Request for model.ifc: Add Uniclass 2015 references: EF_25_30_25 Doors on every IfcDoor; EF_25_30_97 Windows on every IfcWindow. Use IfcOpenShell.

First a look at what the model holds.

```python
import ifcopenshell

model = ifcopenshell.open("model.ifc")
print(model.schema)
print("classifications:", [c.Name for c in model.by_type("IfcClassification")])
for ifc_class in ("IfcDoor", "IfcRoof", "IfcStair", "IfcWall", "IfcWindow"):
    print(ifc_class, len(model.by_type(ifc_class)))
```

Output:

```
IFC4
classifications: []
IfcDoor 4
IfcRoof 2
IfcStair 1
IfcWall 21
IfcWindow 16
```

```python
import ifcopenshell
import ifcopenshell.api.classification

model = ifcopenshell.open("model.ifc")

system = ifcopenshell.api.classification.add_classification(model, classification="Uniclass 2015")

codes = {
    "IfcDoor": ("EF_25_30_25", "Doors"),
    "IfcWindow": ("EF_25_30_97", "Windows"),
}
for ifc_class, (code, name) in codes.items():
    products = model.by_type(ifc_class)
    ifcopenshell.api.classification.add_reference(
        model, products=products, classification=system, identification=code, name=name
    )
    print(code, len(products))

model.write("model_rev.ifc")
```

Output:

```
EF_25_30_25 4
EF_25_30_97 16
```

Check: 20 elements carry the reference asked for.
